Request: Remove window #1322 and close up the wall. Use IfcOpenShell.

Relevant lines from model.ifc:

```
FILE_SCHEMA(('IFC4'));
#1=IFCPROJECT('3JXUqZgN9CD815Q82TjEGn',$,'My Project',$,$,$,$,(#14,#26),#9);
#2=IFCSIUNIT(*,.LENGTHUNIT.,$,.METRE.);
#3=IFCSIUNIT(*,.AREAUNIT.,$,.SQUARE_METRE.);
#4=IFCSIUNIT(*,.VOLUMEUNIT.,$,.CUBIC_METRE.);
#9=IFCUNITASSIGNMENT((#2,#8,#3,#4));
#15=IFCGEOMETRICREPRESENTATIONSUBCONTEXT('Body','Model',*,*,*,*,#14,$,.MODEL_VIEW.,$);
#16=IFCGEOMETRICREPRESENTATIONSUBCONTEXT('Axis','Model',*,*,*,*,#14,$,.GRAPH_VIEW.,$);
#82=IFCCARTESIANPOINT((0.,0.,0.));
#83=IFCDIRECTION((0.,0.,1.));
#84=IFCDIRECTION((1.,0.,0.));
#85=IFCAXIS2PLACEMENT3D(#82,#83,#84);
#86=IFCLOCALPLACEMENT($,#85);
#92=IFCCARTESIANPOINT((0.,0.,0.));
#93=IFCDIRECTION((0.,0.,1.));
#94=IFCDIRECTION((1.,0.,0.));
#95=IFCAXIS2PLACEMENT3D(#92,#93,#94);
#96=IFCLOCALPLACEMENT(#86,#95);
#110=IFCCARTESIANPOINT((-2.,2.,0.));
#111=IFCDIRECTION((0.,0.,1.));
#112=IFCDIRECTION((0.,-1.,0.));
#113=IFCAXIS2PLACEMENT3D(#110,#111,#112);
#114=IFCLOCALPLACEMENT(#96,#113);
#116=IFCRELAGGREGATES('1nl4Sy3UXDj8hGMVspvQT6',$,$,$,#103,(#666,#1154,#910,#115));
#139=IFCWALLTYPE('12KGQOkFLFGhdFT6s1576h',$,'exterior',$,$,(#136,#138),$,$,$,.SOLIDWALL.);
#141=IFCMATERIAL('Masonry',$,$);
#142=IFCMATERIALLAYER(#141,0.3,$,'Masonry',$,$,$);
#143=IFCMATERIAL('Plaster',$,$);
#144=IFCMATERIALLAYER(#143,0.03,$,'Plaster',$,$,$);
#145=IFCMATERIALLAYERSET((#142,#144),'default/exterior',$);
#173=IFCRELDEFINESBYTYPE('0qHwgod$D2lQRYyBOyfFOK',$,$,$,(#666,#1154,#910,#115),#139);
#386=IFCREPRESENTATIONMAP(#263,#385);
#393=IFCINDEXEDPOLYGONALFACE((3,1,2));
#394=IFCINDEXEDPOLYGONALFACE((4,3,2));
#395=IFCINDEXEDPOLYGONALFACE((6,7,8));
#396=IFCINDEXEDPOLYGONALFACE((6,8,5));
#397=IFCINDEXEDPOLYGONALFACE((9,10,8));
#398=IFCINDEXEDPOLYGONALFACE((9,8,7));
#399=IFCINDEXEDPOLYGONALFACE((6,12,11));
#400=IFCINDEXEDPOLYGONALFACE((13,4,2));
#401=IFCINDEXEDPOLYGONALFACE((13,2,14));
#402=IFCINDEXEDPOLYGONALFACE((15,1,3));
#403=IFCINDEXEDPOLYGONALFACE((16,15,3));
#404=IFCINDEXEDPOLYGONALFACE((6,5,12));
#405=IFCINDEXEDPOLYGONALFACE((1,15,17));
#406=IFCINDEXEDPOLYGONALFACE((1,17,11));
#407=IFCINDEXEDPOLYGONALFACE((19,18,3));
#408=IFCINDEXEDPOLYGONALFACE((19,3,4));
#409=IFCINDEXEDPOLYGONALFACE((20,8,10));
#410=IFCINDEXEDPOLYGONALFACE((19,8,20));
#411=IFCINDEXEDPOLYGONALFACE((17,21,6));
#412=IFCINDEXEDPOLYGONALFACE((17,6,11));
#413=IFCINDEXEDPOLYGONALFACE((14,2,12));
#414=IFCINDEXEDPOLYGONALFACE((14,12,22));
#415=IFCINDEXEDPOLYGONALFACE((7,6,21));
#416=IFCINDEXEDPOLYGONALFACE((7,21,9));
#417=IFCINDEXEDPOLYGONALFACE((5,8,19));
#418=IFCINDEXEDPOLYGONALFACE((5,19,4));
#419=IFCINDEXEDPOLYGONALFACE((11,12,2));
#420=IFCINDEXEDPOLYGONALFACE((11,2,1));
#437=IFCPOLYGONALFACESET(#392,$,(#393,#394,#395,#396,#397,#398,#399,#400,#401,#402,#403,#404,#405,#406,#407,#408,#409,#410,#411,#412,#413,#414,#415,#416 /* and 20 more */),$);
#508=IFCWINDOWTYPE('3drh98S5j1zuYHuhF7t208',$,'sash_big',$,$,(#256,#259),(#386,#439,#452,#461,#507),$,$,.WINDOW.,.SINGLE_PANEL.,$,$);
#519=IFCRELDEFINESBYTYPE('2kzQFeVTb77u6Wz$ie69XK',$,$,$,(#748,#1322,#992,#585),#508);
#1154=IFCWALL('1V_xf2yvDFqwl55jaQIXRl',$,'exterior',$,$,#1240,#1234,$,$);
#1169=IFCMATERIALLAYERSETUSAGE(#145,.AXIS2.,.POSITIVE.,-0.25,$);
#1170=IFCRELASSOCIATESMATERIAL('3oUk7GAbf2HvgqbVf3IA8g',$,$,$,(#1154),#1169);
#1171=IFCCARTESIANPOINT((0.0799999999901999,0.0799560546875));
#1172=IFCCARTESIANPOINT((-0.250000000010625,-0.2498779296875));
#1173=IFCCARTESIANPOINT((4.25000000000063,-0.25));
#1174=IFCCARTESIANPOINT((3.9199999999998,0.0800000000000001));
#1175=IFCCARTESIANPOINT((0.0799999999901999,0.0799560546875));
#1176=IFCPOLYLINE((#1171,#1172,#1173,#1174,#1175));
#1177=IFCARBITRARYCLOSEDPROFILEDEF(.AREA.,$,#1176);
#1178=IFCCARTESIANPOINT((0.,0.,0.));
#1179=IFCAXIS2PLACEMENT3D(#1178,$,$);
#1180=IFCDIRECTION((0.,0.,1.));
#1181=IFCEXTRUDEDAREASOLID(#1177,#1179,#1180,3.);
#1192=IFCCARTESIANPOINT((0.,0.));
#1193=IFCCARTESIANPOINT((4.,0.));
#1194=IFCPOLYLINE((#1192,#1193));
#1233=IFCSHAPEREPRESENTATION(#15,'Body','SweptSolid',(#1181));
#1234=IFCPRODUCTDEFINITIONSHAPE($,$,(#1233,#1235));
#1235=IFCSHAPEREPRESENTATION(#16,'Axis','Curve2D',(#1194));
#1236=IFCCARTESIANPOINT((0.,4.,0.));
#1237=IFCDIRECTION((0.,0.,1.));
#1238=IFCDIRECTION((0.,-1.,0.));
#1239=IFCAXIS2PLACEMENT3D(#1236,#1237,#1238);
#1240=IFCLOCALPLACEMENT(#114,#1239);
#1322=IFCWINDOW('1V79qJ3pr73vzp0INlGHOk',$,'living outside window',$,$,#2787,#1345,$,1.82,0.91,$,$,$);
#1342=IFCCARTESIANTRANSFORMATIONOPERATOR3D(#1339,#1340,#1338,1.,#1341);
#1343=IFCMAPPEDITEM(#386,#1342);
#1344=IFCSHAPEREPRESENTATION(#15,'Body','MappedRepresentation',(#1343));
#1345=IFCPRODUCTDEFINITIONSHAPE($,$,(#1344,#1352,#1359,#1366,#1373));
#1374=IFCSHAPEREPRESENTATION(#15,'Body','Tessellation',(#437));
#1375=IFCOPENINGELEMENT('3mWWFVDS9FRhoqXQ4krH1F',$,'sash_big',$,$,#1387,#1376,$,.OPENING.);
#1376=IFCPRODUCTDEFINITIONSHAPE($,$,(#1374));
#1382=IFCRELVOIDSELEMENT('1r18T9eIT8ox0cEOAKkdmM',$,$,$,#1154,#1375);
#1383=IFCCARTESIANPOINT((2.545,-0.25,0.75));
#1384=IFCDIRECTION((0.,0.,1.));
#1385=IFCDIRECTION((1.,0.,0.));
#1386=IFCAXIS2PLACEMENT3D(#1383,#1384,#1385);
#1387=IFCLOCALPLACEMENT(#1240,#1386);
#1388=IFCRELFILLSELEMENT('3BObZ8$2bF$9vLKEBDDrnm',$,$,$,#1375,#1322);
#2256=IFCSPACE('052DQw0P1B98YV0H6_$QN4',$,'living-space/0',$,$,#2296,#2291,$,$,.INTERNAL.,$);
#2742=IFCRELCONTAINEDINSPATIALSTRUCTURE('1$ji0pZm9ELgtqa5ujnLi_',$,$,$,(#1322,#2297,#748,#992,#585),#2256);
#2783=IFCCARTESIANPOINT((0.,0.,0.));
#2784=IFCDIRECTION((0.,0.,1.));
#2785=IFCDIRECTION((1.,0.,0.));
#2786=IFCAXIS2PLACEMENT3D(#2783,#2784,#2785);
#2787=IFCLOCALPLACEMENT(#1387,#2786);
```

```python
import ifcopenshell
import ifcopenshell.api.feature
import ifcopenshell.api.root
import ifcopenshell.geom
import ifcopenshell.util.shape

model = ifcopenshell.open("model.ifc")
settings = ifcopenshell.geom.settings()


def volume(element):
    """Net volume in cubic metres, openings subtracted."""
    shape = ifcopenshell.geom.create_shape(settings, element)
    return ifcopenshell.util.shape.get_volume(shape.geometry)


window = model.by_id(1322)
opening = window.FillsVoids[0].RelatingOpeningElement
wall = opening.VoidsElements[0].RelatingBuildingElement
before = volume(wall)

ifcopenshell.api.root.remove_product(model, product=window)
ifcopenshell.api.feature.remove_feature(model, feature=opening)

after = volume(wall)

print(f"wall volume {before:.3f} -> {after:.3f} m3")

model.write("model_rev.ifc")
```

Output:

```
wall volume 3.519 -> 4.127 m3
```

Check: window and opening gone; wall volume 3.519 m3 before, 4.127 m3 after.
